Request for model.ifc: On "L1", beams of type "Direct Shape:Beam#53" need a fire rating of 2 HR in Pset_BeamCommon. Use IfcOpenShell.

First a look at what the model holds.

```python
import ifcopenshell
import ifcopenshell.util.element

model = ifcopenshell.open("model.ifc")
print(model.schema)
storey = next(s for s in model.by_type("IfcBuildingStorey") if s.Name == "L1")
beams = [e for e in ifcopenshell.util.element.get_decomposition(storey) if e.is_a("IfcBeam")]
seen = {}
for e in beams:
    element_type = ifcopenshell.util.element.get_type(e)
    key = (element_type.Name if element_type != e and element_type else None, ifcopenshell.util.element.get_pset(e, "Pset_BeamCommon", "FireRating"))
    seen[key] = seen.get(key, 0) + 1
for (name, value), count in sorted(seen.items(), key=str):
    print(count, "x", name, "|", value)
```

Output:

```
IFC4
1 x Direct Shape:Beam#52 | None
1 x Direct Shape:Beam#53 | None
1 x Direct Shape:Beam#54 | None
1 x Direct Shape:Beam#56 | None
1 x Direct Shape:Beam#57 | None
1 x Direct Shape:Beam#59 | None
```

```python
import ifcopenshell
import ifcopenshell.api.pset
import ifcopenshell.util.element

model = ifcopenshell.open("model.ifc")

storey = next(s for s in model.by_type("IfcBuildingStorey") if s.Name == "L1")
beams = [e for e in ifcopenshell.util.element.get_decomposition(storey) if e.is_a("IfcBeam")]

count = 0
for e in beams:
    element_type = ifcopenshell.util.element.get_type(e)
    if element_type in (None, e) or element_type.Name != "Direct Shape:Beam#53":
        continue
    # add_pset returns the element's existing set when there is one.
    pset = ifcopenshell.api.pset.add_pset(model, product=e, name="Pset_BeamCommon")
    ifcopenshell.api.pset.edit_pset(model, pset=pset, properties={"FireRating": "2 HR"})
    count += 1

print(count, "beams updated")

model.write("model_edited.ifc")
```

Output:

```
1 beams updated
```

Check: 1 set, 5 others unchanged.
